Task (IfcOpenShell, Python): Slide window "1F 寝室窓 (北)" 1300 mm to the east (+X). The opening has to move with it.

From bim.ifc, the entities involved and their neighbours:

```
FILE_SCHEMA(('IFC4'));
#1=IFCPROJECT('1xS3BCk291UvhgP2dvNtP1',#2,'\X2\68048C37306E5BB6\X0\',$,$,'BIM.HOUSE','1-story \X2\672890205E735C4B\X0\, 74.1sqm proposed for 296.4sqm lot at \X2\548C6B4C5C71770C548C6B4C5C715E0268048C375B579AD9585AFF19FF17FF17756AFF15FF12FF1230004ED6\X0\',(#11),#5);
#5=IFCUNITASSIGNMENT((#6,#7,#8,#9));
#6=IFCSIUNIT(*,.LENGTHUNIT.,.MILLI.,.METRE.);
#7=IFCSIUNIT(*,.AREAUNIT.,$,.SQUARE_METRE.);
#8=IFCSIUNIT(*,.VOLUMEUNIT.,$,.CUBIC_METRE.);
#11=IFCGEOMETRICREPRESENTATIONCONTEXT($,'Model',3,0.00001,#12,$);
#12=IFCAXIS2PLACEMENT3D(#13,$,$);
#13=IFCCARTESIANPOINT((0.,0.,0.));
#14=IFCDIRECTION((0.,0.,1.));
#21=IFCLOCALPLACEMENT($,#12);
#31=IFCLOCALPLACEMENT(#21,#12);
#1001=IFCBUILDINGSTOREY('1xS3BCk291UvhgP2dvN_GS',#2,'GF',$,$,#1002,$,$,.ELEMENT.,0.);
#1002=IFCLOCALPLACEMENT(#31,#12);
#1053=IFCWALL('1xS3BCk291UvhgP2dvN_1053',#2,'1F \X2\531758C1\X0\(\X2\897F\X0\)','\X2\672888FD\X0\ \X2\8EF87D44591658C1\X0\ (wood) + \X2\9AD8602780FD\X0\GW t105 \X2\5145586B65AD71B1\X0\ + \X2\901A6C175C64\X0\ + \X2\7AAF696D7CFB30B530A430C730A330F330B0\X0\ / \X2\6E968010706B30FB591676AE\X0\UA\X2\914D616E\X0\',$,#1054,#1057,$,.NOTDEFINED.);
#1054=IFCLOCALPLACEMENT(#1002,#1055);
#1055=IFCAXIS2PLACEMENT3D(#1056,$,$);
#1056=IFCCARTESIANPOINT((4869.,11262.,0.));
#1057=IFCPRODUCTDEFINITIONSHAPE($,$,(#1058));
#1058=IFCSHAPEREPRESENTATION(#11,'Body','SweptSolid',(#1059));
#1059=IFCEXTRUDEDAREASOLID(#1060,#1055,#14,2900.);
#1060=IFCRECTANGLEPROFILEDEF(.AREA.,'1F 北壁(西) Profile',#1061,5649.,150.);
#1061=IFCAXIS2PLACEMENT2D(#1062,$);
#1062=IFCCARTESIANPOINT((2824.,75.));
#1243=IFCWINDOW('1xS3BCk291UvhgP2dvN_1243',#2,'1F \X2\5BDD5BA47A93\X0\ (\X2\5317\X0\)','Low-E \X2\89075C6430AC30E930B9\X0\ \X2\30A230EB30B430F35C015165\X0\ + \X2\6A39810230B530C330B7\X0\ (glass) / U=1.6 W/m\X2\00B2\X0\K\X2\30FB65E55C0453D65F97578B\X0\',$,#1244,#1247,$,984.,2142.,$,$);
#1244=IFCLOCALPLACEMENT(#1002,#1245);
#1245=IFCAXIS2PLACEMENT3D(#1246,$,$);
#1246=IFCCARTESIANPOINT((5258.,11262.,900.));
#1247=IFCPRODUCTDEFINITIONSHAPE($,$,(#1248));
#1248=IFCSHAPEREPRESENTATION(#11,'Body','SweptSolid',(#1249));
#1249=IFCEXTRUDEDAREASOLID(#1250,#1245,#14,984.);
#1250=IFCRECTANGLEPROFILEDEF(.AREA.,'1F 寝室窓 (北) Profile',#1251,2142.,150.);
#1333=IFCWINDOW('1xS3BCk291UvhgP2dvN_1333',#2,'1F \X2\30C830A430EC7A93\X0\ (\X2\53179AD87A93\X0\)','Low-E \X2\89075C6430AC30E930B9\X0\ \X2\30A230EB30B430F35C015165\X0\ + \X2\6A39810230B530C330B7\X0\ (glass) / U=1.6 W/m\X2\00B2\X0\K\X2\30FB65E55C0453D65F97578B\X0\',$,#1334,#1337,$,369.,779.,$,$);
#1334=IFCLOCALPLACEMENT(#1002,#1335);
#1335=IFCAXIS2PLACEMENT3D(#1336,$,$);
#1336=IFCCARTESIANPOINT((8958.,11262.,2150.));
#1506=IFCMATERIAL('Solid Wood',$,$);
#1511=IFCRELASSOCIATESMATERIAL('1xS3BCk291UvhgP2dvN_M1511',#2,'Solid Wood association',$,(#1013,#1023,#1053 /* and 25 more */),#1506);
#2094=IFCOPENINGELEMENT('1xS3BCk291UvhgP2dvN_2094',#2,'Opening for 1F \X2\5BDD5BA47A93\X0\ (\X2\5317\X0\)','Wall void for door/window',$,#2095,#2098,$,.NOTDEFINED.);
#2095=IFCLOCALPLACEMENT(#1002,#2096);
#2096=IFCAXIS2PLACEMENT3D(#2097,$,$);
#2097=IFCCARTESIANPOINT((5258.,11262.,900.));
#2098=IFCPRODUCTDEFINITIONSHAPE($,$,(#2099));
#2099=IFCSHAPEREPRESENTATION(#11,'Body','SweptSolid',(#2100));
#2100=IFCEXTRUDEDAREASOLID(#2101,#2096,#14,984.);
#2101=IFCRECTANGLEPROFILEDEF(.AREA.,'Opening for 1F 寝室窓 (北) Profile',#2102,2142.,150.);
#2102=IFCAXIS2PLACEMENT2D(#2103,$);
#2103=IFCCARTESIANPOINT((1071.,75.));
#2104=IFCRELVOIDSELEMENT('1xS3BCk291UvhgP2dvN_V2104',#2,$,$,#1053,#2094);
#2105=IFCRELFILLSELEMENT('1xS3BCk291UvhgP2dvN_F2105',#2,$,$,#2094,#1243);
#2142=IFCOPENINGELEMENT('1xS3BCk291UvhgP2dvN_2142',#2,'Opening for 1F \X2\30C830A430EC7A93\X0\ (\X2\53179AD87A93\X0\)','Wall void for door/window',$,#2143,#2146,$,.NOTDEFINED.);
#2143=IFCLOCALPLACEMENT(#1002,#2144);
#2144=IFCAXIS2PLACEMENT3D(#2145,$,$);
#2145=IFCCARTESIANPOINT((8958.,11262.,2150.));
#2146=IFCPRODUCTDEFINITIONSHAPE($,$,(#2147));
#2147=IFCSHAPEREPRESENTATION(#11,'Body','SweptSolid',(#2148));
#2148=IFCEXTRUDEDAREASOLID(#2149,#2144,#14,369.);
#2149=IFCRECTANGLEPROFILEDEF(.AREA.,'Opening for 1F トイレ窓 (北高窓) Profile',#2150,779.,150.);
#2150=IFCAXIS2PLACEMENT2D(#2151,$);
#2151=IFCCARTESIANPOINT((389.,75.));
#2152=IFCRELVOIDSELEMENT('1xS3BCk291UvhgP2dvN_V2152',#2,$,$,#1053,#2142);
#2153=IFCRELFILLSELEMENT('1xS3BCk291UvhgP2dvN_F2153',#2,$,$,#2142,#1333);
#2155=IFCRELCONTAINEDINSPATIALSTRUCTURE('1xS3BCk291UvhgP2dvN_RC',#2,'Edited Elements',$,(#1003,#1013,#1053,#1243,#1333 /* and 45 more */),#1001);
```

```python
import ifcopenshell
import ifcopenshell.api.geometry
import ifcopenshell.util.placement

model = ifcopenshell.open("bim.ifc")

window = model.by_guid("1xS3BCk291UvhgP2dvN_1243")
opening = window.FillsVoids[0].RelatingOpeningElement
wall = opening.VoidsElements[0].RelatingBuildingElement

wall_matrix = ifcopenshell.util.placement.get_local_placement(wall.ObjectPlacement)
shift = wall_matrix[:3, 0] * 1300.0
before = ifcopenshell.util.placement.get_local_placement(window.ObjectPlacement)[:3, 3].copy()

# The window is not placed relative to its opening, so move both.
for product in (opening, window):
    matrix = ifcopenshell.util.placement.get_local_placement(product.ObjectPlacement)
    matrix[:3, 3] += shift
    ifcopenshell.api.geometry.edit_object_placement(model, product=product, matrix=matrix, is_si=False)

after = ifcopenshell.util.placement.get_local_placement(window.ObjectPlacement)[:3, 3]
print("window moved by", (after - before).round(3) + 0.0)

model.write("bim_rev.ifc")
```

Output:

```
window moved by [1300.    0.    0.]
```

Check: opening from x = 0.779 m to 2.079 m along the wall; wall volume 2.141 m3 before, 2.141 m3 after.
